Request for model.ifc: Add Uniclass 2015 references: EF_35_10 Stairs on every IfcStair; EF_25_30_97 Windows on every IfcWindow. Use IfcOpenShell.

First a look at what the model holds.

```python
import ifcopenshell

model = ifcopenshell.open("model.ifc")
print(model.schema)
print("classifications:", [c.Name for c in model.by_type("IfcClassification")])
for ifc_class in ("IfcDoor", "IfcRoof", "IfcStair", "IfcWall", "IfcWindow"):
    print(ifc_class, len(model.by_type(ifc_class)))
```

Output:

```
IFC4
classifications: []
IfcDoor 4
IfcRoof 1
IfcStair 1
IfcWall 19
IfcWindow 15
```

```python
import ifcopenshell
import ifcopenshell.api.classification

model = ifcopenshell.open("model.ifc")

system = ifcopenshell.api.classification.add_classification(model, classification="Uniclass 2015")

codes = {
    "IfcStair": ("EF_35_10", "Stairs"),
    "IfcWindow": ("EF_25_30_97", "Windows"),
}
for ifc_class, (code, name) in codes.items():
    products = model.by_type(ifc_class)
    ifcopenshell.api.classification.add_reference(
        model, products=products, classification=system, identification=code, name=name
    )
    print(code, len(products))

model.write("model-out.ifc")
```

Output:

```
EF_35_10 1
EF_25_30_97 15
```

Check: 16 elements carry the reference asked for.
